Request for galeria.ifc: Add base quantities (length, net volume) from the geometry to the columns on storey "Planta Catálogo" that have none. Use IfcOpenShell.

First a look at what the model holds.

```python
import ifcopenshell
import ifcopenshell.util.element
import ifcopenshell.util.unit

model = ifcopenshell.open("galeria.ifc")
print(model.schema)
for unit_type in ("LENGTHUNIT", "AREAUNIT", "VOLUMEUNIT"):
    print(unit_type, ifcopenshell.util.unit.calculate_unit_scale(model, unit_type))
storey = next(s for s in model.by_type("IfcBuildingStorey") if s.Name == "Planta Catálogo")
columns = [e for e in ifcopenshell.util.element.get_decomposition(storey) if e.is_a("IfcColumn")]
for e in sorted(columns, key=lambda e: e.id()):
    print(e.id(), e.is_a(), e.Name, list(ifcopenshell.util.element.get_psets(e, qtos_only=True)), sep=" | ")
```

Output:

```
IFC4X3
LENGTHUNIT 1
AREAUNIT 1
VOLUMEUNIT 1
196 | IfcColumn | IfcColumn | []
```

```python
import ifcopenshell
import ifcopenshell.api.pset
import ifcopenshell.geom
import ifcopenshell.util.element
import ifcopenshell.util.shape
import ifcopenshell.util.unit

model = ifcopenshell.open("galeria.ifc")
unit_scale = ifcopenshell.util.unit.calculate_unit_scale(model)
volume_scale = ifcopenshell.util.unit.calculate_unit_scale(model, "VOLUMEUNIT")
settings = ifcopenshell.geom.settings()

storey = next(s for s in model.by_type("IfcBuildingStorey") if s.Name == "Planta Catálogo")
columns = [e for e in ifcopenshell.util.element.get_decomposition(storey) if e.is_a("IfcColumn")]

for e in sorted(columns, key=lambda e: e.id()):
    if ifcopenshell.util.element.get_psets(e, qtos_only=True, should_inherit=False):
        continue
    # Geometry comes back in metres, in the element's own axes.
    shape = ifcopenshell.geom.create_shape(settings, e)
    values = {
        "Length": ifcopenshell.util.shape.get_z(shape.geometry) / unit_scale,
        "NetVolume": ifcopenshell.util.shape.get_volume(shape.geometry) / volume_scale,
    }
    qto = ifcopenshell.api.pset.add_qto(model, product=e, name="Qto_ColumnBaseQuantities")
    ifcopenshell.api.pset.edit_qto(model, qto=qto, properties=values)
    print(e.id(), {k: round(v, 3) for k, v in values.items()})

model.write("galeria_updated.ifc")
```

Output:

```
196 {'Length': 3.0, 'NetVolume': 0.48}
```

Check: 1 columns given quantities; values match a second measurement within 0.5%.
